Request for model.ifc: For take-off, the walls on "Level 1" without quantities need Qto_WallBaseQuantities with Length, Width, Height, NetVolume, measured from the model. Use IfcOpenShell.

First a look at what the model holds.

```python
import ifcopenshell
import ifcopenshell.util.element
import ifcopenshell.util.unit

model = ifcopenshell.open("model.ifc")
print(model.schema)
for unit_type in ("LENGTHUNIT", "AREAUNIT", "VOLUMEUNIT"):
    print(unit_type, ifcopenshell.util.unit.calculate_unit_scale(model, unit_type))
storey = next(s for s in model.by_type("IfcBuildingStorey") if s.Name == "Level 1")
walls = [e for e in ifcopenshell.util.element.get_decomposition(storey) if e.is_a("IfcWall")]
for e in sorted(walls, key=lambda e: e.id()):
    print(e.id(), e.is_a(), e.Name, list(ifcopenshell.util.element.get_psets(e, qtos_only=True)), sep=" | ")
```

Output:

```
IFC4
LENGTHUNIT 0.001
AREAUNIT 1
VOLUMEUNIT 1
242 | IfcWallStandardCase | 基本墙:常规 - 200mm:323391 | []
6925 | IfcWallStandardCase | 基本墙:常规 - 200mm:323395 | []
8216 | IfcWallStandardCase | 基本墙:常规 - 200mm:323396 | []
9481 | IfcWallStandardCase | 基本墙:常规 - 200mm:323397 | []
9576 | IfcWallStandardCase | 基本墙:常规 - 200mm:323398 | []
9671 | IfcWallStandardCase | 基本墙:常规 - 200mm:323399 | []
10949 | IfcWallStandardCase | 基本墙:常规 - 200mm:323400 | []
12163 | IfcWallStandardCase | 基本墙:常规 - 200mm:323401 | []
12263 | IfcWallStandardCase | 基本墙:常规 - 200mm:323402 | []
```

```python
import ifcopenshell
import ifcopenshell.api.pset
import ifcopenshell.geom
import ifcopenshell.util.element
import ifcopenshell.util.shape
import ifcopenshell.util.unit

model = ifcopenshell.open("model.ifc")
unit_scale = ifcopenshell.util.unit.calculate_unit_scale(model)
volume_scale = ifcopenshell.util.unit.calculate_unit_scale(model, "VOLUMEUNIT")
settings = ifcopenshell.geom.settings()

storey = next(s for s in model.by_type("IfcBuildingStorey") if s.Name == "Level 1")
walls = [e for e in ifcopenshell.util.element.get_decomposition(storey) if e.is_a("IfcWall")]

for e in sorted(walls, key=lambda e: e.id()):
    if ifcopenshell.util.element.get_psets(e, qtos_only=True, should_inherit=False):
        continue
    # Geometry comes back in metres, in the element's own axes.
    shape = ifcopenshell.geom.create_shape(settings, e)
    values = {
        "Length": ifcopenshell.util.shape.get_x(shape.geometry) / unit_scale,
        "Width": ifcopenshell.util.shape.get_y(shape.geometry) / unit_scale,
        "Height": ifcopenshell.util.shape.get_z(shape.geometry) / unit_scale,
        "NetVolume": ifcopenshell.util.shape.get_volume(shape.geometry) / volume_scale,
    }
    qto = ifcopenshell.api.pset.add_qto(model, product=e, name="Qto_WallBaseQuantities")
    ifcopenshell.api.pset.edit_qto(model, qto=qto, properties=values)
    print(e.id(), {k: round(v, 3) for k, v in values.items()})

model.write("model_v2.ifc")
```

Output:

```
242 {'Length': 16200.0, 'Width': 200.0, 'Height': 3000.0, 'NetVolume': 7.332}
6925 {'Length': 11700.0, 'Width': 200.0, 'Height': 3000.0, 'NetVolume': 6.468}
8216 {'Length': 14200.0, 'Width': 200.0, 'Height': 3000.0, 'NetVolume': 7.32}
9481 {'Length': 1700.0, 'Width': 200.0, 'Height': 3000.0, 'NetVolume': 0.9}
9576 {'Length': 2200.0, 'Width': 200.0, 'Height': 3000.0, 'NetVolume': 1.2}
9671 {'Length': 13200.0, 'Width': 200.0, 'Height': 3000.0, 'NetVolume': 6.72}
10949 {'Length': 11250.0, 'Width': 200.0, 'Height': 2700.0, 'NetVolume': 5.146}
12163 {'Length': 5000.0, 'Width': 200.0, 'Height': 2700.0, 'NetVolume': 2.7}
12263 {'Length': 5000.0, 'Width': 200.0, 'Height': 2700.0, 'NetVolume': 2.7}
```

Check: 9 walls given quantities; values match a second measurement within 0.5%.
